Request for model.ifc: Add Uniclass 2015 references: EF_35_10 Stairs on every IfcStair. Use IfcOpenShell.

First a look at what the model holds.

```python
import ifcopenshell

model = ifcopenshell.open("model.ifc")
print(model.schema)
print("classifications:", [c.Name for c in model.by_type("IfcClassification")])
for ifc_class in ("IfcDoor", "IfcRoof", "IfcStair", "IfcWall", "IfcWindow"):
    print(ifc_class, len(model.by_type(ifc_class)))
```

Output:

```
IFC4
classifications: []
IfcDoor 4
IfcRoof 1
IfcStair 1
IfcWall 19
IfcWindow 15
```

```python
import ifcopenshell
import ifcopenshell.api.classification

model = ifcopenshell.open("model.ifc")

system = ifcopenshell.api.classification.add_classification(model, classification="Uniclass 2015")

codes = {
    "IfcStair": ("EF_35_10", "Stairs"),
}
for ifc_class, (code, name) in codes.items():
    products = model.by_type(ifc_class)
    ifcopenshell.api.classification.add_reference(
        model, products=products, classification=system, identification=code, name=name
    )
    print(code, len(products))

model.write("model_updated.ifc")
```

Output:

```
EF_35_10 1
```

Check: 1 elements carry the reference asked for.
